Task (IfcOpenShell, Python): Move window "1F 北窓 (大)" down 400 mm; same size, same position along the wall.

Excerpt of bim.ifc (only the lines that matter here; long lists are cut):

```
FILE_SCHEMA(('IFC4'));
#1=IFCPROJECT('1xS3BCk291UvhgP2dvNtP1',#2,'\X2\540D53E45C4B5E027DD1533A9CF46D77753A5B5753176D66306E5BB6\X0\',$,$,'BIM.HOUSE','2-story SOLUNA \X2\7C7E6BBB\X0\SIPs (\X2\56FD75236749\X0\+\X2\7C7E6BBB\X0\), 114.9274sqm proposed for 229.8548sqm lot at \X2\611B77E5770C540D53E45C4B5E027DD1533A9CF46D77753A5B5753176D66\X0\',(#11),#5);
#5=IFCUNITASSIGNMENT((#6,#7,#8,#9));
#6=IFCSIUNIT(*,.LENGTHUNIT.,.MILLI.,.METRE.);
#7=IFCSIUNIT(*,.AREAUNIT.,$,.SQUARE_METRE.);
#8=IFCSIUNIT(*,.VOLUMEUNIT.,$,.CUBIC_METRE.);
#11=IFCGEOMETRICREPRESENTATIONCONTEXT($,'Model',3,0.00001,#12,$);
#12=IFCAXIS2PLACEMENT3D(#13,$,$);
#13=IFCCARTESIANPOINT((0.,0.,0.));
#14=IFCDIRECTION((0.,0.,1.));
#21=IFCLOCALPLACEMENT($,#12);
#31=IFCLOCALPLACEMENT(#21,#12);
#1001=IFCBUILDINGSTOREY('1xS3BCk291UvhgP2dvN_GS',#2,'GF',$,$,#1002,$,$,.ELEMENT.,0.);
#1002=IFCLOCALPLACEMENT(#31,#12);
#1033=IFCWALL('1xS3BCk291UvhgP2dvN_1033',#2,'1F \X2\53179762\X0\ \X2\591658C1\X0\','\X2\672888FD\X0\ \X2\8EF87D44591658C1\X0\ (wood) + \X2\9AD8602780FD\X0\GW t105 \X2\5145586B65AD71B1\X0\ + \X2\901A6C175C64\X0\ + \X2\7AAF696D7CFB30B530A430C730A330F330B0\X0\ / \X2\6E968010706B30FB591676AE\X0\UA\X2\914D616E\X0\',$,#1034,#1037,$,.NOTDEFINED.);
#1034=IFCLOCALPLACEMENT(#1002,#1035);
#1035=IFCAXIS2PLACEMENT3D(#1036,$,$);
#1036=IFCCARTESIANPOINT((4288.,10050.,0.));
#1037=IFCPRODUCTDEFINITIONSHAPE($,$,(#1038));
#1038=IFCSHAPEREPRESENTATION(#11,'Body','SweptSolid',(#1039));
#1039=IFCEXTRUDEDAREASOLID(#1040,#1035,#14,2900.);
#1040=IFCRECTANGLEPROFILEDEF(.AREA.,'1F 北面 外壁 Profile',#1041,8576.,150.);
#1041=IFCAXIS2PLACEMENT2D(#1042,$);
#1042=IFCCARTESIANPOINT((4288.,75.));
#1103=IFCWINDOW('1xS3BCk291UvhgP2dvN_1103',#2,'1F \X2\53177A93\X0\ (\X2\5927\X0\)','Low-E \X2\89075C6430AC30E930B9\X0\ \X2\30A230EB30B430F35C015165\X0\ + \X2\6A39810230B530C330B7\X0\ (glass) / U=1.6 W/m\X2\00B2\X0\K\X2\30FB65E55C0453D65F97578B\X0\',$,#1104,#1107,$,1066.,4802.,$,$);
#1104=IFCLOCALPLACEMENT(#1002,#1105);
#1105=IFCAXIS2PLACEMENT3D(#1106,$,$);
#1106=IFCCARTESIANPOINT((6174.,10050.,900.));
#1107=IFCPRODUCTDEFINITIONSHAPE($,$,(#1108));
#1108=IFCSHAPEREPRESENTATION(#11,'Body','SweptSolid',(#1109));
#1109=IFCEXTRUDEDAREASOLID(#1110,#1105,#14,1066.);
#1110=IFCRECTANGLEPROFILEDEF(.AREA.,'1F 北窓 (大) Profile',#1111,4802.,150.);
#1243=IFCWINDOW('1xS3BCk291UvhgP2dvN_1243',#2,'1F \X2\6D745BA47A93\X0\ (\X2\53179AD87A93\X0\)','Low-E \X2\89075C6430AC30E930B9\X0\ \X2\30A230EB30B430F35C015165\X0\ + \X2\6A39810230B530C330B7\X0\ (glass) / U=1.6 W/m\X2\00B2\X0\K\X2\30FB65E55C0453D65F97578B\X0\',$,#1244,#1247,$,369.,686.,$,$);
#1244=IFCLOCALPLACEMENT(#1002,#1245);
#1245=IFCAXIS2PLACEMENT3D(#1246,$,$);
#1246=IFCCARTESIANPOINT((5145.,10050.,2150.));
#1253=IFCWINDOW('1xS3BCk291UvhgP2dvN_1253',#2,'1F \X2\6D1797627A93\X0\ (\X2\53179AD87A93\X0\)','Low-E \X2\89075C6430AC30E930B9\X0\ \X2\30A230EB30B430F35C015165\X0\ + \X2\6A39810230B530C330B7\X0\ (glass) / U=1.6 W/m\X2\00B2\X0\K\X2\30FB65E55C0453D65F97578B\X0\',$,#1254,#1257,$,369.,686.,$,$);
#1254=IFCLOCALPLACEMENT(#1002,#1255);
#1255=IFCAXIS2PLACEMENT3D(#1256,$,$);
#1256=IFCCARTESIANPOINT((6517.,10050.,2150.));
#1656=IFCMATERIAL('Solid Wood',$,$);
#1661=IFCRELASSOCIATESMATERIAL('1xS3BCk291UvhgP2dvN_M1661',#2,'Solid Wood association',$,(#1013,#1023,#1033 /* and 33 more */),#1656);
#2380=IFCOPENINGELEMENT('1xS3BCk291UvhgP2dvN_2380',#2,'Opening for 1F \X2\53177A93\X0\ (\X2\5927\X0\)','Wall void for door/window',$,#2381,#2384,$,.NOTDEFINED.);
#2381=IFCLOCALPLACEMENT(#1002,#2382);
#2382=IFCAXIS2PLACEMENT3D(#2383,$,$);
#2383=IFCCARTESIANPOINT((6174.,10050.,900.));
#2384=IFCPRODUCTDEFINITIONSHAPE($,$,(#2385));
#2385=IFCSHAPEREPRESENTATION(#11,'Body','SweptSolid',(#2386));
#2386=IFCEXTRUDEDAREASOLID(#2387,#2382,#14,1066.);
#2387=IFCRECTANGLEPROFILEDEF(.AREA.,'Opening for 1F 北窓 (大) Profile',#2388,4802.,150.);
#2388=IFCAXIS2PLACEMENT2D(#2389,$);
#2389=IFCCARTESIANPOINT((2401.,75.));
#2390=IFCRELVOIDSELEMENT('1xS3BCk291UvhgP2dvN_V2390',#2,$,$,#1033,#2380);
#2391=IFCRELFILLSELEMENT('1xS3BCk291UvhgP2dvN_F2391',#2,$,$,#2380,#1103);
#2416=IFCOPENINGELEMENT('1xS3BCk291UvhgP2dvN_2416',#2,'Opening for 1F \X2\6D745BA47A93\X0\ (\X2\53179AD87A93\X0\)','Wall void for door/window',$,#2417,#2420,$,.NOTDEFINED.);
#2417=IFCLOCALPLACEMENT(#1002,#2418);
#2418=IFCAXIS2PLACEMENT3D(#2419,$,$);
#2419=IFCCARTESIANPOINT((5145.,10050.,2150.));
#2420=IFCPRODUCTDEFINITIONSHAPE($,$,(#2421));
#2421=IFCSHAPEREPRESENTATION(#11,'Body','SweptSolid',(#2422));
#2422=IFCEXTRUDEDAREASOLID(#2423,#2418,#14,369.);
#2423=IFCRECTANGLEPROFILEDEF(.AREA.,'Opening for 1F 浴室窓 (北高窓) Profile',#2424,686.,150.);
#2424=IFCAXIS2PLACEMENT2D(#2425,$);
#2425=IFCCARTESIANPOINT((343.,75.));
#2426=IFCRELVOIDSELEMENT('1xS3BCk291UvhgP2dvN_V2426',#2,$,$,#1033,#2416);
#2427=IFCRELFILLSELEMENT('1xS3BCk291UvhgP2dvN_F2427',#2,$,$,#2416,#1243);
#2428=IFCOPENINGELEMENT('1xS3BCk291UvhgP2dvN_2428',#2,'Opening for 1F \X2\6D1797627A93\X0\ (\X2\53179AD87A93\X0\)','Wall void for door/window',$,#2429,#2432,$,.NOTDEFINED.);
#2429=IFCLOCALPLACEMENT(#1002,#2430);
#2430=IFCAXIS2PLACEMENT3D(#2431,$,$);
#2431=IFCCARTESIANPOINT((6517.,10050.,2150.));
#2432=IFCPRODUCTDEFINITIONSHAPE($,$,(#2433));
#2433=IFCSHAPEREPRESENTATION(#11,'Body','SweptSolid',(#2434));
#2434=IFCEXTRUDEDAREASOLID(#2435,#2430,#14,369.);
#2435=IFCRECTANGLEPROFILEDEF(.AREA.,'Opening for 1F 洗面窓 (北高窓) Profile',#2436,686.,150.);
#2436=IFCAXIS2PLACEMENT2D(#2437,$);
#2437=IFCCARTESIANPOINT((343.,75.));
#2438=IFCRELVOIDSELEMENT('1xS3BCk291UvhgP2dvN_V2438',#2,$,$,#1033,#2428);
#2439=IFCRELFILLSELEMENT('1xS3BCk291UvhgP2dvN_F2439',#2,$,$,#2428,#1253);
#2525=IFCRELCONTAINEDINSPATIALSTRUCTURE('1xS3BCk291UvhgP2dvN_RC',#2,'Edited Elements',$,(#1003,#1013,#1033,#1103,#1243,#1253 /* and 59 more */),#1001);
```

```python
import numpy as np
import ifcopenshell
import ifcopenshell.api.geometry
import ifcopenshell.util.placement
import ifcopenshell.util.unit

model = ifcopenshell.open("bim.ifc")
unit_scale = ifcopenshell.util.unit.calculate_unit_scale(model)

window = model.by_guid("1xS3BCk291UvhgP2dvN_1103")
opening = window.FillsVoids[0].RelatingOpeningElement
dz = -400.0

shift = np.array([0.0, 0.0, dz])
# The window is not placed relative to its opening, so move both.
for product in (opening, window):
    matrix = ifcopenshell.util.placement.get_local_placement(product.ObjectPlacement)
    matrix[:3, 3] += shift
    ifcopenshell.api.geometry.edit_object_placement(model, product=product, matrix=matrix, is_si=False)

print(f"moved by {dz * unit_scale:+.3f} m")

model.write("bim_v2.ifc")
```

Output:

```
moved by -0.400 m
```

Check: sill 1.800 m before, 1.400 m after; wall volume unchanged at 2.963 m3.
